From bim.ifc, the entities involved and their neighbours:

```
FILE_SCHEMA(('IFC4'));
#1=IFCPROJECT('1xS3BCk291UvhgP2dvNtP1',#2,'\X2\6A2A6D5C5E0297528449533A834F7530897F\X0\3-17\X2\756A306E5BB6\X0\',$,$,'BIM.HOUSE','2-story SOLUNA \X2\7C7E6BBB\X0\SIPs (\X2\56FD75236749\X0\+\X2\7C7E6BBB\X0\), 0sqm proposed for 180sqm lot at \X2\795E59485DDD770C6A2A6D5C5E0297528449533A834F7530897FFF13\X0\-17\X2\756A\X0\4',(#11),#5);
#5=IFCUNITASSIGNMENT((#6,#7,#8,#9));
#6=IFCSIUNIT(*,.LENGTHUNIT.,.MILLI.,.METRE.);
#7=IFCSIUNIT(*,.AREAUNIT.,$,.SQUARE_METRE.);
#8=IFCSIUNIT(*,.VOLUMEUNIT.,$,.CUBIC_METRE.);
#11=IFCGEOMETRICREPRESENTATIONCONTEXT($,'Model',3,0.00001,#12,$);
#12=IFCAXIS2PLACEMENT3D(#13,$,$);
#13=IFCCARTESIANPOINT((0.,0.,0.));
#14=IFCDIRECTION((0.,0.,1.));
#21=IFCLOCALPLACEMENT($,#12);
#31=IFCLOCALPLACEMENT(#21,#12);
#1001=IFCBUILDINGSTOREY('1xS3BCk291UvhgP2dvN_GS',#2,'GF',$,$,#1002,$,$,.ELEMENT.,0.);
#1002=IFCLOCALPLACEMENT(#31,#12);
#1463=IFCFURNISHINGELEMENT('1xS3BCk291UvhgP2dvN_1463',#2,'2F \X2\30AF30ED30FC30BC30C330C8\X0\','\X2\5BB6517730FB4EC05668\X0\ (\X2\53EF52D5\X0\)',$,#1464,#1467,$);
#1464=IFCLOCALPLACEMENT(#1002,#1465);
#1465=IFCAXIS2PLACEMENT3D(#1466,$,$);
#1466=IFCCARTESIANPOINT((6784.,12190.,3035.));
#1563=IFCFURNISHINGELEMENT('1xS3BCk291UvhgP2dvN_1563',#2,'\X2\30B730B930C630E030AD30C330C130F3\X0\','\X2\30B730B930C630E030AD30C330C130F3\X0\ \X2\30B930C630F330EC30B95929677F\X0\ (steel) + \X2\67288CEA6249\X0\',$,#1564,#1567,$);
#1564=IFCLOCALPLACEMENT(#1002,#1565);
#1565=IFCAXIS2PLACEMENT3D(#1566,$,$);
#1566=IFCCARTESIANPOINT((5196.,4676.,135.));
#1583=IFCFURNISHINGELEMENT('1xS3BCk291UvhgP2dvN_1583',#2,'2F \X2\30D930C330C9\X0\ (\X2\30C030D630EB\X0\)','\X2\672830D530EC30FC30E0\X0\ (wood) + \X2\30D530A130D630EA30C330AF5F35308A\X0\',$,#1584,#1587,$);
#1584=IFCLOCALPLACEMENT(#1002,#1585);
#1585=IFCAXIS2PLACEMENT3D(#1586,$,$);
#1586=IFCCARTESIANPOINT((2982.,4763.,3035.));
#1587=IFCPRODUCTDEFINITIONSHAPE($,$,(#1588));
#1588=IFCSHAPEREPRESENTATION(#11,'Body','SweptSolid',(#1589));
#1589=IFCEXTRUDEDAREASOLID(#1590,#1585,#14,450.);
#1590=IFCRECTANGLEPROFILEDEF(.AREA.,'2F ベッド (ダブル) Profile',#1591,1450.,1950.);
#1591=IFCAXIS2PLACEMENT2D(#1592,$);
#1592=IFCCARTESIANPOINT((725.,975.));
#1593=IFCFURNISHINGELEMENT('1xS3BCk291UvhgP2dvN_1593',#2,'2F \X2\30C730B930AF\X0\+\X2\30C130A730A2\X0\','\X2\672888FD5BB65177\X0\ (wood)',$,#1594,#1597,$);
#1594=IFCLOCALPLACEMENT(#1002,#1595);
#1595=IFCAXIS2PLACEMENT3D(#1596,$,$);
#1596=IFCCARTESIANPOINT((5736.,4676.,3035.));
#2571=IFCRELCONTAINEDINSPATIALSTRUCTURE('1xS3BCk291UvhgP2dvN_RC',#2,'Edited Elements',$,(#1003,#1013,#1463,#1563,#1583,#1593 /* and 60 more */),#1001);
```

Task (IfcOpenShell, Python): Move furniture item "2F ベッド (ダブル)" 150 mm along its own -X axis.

```python
import ifcopenshell
import ifcopenshell.api.geometry
import ifcopenshell.util.placement
import ifcopenshell.util.unit

model = ifcopenshell.open("bim.ifc")
unit_scale = ifcopenshell.util.unit.calculate_unit_scale(model)

item = model.by_guid("1xS3BCk291UvhgP2dvN_1583")
matrix = ifcopenshell.util.placement.get_local_placement(item.ObjectPlacement)
matrix[:3, 3] -= matrix[:3, 0] * 0.15 / unit_scale
ifcopenshell.api.geometry.edit_object_placement(model, product=item, matrix=matrix, is_si=False)

print(ifcopenshell.util.placement.get_local_placement(item.ObjectPlacement).round(3) + 0.0)

model.write("bim_updated.ifc")
```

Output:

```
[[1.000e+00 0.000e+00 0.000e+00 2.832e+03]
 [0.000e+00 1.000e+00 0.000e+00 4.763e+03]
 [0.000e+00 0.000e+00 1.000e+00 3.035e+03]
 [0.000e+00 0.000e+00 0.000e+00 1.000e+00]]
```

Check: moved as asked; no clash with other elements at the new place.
